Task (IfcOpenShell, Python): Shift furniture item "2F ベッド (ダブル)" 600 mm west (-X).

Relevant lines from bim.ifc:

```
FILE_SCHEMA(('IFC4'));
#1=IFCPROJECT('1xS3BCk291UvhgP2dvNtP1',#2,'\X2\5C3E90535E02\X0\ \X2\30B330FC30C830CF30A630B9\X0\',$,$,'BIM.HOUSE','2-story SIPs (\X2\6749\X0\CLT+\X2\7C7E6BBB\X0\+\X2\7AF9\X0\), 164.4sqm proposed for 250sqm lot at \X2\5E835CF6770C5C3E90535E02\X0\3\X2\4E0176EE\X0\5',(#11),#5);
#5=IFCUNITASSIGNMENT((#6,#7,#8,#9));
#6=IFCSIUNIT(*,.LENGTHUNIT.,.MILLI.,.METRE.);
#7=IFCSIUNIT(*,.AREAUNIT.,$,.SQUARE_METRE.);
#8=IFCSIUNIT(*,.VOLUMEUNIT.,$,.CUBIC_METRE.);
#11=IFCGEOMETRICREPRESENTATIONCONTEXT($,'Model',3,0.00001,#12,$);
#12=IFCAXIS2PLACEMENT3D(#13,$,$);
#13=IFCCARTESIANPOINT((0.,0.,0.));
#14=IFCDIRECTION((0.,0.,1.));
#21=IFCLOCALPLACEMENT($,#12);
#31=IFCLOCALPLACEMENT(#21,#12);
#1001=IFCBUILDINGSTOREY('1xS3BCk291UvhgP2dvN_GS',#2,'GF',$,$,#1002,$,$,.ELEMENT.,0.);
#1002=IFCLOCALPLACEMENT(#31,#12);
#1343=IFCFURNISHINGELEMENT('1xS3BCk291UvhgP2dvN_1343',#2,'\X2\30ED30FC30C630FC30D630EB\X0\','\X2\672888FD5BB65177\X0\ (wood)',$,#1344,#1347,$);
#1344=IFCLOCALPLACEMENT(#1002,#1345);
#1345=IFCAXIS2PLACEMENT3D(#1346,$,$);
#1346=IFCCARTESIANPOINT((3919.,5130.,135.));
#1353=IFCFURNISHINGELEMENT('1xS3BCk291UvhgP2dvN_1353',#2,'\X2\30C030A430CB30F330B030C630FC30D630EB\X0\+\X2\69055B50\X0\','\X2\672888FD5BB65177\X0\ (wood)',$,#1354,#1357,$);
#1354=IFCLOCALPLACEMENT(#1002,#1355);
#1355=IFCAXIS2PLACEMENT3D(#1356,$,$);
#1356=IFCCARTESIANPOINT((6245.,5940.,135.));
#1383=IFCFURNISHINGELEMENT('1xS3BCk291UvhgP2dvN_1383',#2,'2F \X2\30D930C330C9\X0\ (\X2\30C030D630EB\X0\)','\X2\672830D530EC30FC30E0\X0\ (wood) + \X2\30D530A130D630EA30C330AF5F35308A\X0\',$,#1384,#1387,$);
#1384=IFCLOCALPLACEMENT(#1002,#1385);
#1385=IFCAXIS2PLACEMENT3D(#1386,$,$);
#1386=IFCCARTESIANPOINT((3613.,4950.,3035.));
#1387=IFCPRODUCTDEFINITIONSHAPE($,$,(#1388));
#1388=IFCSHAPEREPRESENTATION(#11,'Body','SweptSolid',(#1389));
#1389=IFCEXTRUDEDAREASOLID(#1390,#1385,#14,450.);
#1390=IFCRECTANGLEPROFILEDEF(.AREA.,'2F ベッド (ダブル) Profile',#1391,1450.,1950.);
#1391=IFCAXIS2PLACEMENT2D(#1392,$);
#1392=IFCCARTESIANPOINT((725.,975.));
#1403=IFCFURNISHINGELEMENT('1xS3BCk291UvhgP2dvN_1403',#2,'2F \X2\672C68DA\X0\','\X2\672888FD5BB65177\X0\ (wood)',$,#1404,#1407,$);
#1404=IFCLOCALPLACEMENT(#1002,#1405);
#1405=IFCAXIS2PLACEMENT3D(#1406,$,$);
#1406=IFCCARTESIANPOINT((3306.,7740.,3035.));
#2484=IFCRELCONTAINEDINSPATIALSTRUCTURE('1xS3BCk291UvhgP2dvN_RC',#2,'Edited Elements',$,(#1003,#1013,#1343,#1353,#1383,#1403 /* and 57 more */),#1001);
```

```python
import ifcopenshell
import ifcopenshell.api.geometry
import ifcopenshell.util.placement
import ifcopenshell.util.unit

model = ifcopenshell.open("bim.ifc")
unit_scale = ifcopenshell.util.unit.calculate_unit_scale(model)

item = model.by_guid("1xS3BCk291UvhgP2dvN_1383")
matrix = ifcopenshell.util.placement.get_local_placement(item.ObjectPlacement)
matrix[0, 3] -= 0.6 / unit_scale
ifcopenshell.api.geometry.edit_object_placement(model, product=item, matrix=matrix, is_si=False)

print(ifcopenshell.util.placement.get_local_placement(item.ObjectPlacement).round(3) + 0.0)

model.write("bim_rev.ifc")
```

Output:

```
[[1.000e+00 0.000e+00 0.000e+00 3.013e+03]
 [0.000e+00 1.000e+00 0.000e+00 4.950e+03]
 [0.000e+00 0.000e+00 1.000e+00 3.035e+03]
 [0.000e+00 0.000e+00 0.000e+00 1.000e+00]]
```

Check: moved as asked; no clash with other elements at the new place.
